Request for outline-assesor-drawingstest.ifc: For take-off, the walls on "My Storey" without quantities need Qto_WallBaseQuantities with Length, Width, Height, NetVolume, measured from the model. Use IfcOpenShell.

First a look at what the model holds.

```python
import ifcopenshell
import ifcopenshell.util.element
import ifcopenshell.util.unit

model = ifcopenshell.open("outline-assesor-drawingstest.ifc")
print(model.schema)
for unit_type in ("LENGTHUNIT", "AREAUNIT", "VOLUMEUNIT"):
    print(unit_type, ifcopenshell.util.unit.calculate_unit_scale(model, unit_type))
storey = next(s for s in model.by_type("IfcBuildingStorey") if s.Name == "My Storey")
walls = [e for e in ifcopenshell.util.element.get_decomposition(storey) if e.is_a("IfcWall")]
for e in sorted(walls, key=lambda e: e.id()):
    print(e.id(), e.is_a(), e.Name, list(ifcopenshell.util.element.get_psets(e, qtos_only=True)), sep=" | ")
```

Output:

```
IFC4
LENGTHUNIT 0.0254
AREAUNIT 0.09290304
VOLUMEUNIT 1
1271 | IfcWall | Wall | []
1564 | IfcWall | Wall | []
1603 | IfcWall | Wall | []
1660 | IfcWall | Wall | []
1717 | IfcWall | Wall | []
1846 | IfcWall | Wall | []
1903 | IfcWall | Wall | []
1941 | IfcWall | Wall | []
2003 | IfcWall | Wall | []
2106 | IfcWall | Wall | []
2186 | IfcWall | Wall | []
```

```python
import ifcopenshell
import ifcopenshell.api.pset
import ifcopenshell.geom
import ifcopenshell.util.element
import ifcopenshell.util.shape
import ifcopenshell.util.unit

model = ifcopenshell.open("outline-assesor-drawingstest.ifc")
unit_scale = ifcopenshell.util.unit.calculate_unit_scale(model)
volume_scale = ifcopenshell.util.unit.calculate_unit_scale(model, "VOLUMEUNIT")
settings = ifcopenshell.geom.settings()

storey = next(s for s in model.by_type("IfcBuildingStorey") if s.Name == "My Storey")
walls = [e for e in ifcopenshell.util.element.get_decomposition(storey) if e.is_a("IfcWall")]

for e in sorted(walls, key=lambda e: e.id()):
    if ifcopenshell.util.element.get_psets(e, qtos_only=True, should_inherit=False):
        continue
    # Geometry comes back in metres, in the element's own axes.
    shape = ifcopenshell.geom.create_shape(settings, e)
    values = {
        "Length": ifcopenshell.util.shape.get_x(shape.geometry) / unit_scale,
        "Width": ifcopenshell.util.shape.get_y(shape.geometry) / unit_scale,
        "Height": ifcopenshell.util.shape.get_z(shape.geometry) / unit_scale,
        "NetVolume": ifcopenshell.util.shape.get_volume(shape.geometry) / volume_scale,
    }
    qto = ifcopenshell.api.pset.add_qto(model, product=e, name="Qto_WallBaseQuantities")
    ifcopenshell.api.pset.edit_qto(model, qto=qto, properties=values)
    print(e.id(), {k: round(v, 3) for k, v in values.items()})

model.write("outline-assesor-drawingstest_updated.ifc")
```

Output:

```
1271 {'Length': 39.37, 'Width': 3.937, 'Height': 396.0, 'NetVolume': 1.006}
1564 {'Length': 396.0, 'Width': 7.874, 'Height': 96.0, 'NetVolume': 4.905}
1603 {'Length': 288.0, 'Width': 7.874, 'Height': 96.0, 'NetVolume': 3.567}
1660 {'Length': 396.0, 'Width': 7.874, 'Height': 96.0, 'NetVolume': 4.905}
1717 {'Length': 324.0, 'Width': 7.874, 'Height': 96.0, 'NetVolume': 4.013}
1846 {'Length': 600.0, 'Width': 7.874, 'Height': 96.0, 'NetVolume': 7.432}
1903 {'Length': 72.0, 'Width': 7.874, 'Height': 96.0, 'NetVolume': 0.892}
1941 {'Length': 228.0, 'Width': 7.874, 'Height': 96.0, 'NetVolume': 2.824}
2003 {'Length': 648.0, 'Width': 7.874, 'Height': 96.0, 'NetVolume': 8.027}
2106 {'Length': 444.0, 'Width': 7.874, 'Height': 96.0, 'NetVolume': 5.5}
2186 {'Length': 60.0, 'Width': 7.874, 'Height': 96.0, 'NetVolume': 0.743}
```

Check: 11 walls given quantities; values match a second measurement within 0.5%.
